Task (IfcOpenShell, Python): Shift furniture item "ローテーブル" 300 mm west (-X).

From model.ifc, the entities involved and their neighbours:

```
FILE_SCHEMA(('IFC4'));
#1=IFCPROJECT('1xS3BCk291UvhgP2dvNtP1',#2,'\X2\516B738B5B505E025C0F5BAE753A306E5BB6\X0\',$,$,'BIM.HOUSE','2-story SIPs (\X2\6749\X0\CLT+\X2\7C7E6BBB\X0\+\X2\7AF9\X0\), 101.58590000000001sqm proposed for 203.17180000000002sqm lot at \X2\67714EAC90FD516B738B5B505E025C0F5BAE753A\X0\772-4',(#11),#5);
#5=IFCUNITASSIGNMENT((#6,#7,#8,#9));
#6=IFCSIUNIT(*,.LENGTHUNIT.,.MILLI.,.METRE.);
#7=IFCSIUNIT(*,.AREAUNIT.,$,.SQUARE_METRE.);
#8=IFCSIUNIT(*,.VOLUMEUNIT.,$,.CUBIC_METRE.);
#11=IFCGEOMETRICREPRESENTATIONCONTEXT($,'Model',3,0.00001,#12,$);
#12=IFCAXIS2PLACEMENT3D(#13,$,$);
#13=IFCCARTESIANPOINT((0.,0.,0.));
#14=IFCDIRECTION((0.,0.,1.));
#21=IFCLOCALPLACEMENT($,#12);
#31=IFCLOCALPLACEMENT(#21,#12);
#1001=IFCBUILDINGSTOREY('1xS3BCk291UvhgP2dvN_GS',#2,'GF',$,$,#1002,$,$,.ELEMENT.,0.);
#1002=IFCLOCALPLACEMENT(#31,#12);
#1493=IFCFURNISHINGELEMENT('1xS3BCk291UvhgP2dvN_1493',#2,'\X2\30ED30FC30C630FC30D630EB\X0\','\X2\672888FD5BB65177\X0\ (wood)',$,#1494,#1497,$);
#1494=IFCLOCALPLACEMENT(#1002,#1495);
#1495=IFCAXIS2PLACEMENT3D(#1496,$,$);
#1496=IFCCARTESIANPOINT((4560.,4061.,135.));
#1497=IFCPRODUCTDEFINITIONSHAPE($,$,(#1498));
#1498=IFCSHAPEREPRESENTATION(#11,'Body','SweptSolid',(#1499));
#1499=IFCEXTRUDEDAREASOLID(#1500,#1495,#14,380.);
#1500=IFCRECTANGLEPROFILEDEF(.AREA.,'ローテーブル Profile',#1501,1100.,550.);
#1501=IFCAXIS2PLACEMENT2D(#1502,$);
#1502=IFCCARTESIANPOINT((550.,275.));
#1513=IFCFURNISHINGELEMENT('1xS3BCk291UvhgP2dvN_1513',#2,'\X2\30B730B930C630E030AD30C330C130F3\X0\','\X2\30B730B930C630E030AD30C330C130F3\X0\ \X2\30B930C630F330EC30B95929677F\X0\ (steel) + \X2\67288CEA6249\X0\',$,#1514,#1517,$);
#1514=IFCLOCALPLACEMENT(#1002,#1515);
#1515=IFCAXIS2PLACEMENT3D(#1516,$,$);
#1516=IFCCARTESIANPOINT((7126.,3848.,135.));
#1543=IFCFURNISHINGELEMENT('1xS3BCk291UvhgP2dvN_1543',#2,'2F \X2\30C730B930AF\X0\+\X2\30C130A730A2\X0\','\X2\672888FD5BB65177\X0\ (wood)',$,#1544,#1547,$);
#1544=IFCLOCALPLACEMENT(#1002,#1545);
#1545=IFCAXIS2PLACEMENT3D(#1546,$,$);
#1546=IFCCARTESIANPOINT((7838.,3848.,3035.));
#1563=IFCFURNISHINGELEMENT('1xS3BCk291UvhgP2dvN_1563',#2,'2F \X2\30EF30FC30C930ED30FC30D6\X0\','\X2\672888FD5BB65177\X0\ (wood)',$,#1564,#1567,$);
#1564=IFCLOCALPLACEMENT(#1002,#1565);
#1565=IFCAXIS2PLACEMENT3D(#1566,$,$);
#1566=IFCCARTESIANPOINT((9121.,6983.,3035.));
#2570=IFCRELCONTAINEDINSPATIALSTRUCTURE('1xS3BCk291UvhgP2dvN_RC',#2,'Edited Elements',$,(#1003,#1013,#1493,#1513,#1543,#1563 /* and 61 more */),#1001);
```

```python
import ifcopenshell
import ifcopenshell.api.geometry
import ifcopenshell.util.placement
import ifcopenshell.util.unit

model = ifcopenshell.open("model.ifc")
unit_scale = ifcopenshell.util.unit.calculate_unit_scale(model)

item = model.by_id(1493)
matrix = ifcopenshell.util.placement.get_local_placement(item.ObjectPlacement)
matrix[0, 3] -= 0.3 / unit_scale
ifcopenshell.api.geometry.edit_object_placement(model, product=item, matrix=matrix, is_si=False)

print(ifcopenshell.util.placement.get_local_placement(item.ObjectPlacement).round(3) + 0.0)

model.write("model_rev.ifc")
```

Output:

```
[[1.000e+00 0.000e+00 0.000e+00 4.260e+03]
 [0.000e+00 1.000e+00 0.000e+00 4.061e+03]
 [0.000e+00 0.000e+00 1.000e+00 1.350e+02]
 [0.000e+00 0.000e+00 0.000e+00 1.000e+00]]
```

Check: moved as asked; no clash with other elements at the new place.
